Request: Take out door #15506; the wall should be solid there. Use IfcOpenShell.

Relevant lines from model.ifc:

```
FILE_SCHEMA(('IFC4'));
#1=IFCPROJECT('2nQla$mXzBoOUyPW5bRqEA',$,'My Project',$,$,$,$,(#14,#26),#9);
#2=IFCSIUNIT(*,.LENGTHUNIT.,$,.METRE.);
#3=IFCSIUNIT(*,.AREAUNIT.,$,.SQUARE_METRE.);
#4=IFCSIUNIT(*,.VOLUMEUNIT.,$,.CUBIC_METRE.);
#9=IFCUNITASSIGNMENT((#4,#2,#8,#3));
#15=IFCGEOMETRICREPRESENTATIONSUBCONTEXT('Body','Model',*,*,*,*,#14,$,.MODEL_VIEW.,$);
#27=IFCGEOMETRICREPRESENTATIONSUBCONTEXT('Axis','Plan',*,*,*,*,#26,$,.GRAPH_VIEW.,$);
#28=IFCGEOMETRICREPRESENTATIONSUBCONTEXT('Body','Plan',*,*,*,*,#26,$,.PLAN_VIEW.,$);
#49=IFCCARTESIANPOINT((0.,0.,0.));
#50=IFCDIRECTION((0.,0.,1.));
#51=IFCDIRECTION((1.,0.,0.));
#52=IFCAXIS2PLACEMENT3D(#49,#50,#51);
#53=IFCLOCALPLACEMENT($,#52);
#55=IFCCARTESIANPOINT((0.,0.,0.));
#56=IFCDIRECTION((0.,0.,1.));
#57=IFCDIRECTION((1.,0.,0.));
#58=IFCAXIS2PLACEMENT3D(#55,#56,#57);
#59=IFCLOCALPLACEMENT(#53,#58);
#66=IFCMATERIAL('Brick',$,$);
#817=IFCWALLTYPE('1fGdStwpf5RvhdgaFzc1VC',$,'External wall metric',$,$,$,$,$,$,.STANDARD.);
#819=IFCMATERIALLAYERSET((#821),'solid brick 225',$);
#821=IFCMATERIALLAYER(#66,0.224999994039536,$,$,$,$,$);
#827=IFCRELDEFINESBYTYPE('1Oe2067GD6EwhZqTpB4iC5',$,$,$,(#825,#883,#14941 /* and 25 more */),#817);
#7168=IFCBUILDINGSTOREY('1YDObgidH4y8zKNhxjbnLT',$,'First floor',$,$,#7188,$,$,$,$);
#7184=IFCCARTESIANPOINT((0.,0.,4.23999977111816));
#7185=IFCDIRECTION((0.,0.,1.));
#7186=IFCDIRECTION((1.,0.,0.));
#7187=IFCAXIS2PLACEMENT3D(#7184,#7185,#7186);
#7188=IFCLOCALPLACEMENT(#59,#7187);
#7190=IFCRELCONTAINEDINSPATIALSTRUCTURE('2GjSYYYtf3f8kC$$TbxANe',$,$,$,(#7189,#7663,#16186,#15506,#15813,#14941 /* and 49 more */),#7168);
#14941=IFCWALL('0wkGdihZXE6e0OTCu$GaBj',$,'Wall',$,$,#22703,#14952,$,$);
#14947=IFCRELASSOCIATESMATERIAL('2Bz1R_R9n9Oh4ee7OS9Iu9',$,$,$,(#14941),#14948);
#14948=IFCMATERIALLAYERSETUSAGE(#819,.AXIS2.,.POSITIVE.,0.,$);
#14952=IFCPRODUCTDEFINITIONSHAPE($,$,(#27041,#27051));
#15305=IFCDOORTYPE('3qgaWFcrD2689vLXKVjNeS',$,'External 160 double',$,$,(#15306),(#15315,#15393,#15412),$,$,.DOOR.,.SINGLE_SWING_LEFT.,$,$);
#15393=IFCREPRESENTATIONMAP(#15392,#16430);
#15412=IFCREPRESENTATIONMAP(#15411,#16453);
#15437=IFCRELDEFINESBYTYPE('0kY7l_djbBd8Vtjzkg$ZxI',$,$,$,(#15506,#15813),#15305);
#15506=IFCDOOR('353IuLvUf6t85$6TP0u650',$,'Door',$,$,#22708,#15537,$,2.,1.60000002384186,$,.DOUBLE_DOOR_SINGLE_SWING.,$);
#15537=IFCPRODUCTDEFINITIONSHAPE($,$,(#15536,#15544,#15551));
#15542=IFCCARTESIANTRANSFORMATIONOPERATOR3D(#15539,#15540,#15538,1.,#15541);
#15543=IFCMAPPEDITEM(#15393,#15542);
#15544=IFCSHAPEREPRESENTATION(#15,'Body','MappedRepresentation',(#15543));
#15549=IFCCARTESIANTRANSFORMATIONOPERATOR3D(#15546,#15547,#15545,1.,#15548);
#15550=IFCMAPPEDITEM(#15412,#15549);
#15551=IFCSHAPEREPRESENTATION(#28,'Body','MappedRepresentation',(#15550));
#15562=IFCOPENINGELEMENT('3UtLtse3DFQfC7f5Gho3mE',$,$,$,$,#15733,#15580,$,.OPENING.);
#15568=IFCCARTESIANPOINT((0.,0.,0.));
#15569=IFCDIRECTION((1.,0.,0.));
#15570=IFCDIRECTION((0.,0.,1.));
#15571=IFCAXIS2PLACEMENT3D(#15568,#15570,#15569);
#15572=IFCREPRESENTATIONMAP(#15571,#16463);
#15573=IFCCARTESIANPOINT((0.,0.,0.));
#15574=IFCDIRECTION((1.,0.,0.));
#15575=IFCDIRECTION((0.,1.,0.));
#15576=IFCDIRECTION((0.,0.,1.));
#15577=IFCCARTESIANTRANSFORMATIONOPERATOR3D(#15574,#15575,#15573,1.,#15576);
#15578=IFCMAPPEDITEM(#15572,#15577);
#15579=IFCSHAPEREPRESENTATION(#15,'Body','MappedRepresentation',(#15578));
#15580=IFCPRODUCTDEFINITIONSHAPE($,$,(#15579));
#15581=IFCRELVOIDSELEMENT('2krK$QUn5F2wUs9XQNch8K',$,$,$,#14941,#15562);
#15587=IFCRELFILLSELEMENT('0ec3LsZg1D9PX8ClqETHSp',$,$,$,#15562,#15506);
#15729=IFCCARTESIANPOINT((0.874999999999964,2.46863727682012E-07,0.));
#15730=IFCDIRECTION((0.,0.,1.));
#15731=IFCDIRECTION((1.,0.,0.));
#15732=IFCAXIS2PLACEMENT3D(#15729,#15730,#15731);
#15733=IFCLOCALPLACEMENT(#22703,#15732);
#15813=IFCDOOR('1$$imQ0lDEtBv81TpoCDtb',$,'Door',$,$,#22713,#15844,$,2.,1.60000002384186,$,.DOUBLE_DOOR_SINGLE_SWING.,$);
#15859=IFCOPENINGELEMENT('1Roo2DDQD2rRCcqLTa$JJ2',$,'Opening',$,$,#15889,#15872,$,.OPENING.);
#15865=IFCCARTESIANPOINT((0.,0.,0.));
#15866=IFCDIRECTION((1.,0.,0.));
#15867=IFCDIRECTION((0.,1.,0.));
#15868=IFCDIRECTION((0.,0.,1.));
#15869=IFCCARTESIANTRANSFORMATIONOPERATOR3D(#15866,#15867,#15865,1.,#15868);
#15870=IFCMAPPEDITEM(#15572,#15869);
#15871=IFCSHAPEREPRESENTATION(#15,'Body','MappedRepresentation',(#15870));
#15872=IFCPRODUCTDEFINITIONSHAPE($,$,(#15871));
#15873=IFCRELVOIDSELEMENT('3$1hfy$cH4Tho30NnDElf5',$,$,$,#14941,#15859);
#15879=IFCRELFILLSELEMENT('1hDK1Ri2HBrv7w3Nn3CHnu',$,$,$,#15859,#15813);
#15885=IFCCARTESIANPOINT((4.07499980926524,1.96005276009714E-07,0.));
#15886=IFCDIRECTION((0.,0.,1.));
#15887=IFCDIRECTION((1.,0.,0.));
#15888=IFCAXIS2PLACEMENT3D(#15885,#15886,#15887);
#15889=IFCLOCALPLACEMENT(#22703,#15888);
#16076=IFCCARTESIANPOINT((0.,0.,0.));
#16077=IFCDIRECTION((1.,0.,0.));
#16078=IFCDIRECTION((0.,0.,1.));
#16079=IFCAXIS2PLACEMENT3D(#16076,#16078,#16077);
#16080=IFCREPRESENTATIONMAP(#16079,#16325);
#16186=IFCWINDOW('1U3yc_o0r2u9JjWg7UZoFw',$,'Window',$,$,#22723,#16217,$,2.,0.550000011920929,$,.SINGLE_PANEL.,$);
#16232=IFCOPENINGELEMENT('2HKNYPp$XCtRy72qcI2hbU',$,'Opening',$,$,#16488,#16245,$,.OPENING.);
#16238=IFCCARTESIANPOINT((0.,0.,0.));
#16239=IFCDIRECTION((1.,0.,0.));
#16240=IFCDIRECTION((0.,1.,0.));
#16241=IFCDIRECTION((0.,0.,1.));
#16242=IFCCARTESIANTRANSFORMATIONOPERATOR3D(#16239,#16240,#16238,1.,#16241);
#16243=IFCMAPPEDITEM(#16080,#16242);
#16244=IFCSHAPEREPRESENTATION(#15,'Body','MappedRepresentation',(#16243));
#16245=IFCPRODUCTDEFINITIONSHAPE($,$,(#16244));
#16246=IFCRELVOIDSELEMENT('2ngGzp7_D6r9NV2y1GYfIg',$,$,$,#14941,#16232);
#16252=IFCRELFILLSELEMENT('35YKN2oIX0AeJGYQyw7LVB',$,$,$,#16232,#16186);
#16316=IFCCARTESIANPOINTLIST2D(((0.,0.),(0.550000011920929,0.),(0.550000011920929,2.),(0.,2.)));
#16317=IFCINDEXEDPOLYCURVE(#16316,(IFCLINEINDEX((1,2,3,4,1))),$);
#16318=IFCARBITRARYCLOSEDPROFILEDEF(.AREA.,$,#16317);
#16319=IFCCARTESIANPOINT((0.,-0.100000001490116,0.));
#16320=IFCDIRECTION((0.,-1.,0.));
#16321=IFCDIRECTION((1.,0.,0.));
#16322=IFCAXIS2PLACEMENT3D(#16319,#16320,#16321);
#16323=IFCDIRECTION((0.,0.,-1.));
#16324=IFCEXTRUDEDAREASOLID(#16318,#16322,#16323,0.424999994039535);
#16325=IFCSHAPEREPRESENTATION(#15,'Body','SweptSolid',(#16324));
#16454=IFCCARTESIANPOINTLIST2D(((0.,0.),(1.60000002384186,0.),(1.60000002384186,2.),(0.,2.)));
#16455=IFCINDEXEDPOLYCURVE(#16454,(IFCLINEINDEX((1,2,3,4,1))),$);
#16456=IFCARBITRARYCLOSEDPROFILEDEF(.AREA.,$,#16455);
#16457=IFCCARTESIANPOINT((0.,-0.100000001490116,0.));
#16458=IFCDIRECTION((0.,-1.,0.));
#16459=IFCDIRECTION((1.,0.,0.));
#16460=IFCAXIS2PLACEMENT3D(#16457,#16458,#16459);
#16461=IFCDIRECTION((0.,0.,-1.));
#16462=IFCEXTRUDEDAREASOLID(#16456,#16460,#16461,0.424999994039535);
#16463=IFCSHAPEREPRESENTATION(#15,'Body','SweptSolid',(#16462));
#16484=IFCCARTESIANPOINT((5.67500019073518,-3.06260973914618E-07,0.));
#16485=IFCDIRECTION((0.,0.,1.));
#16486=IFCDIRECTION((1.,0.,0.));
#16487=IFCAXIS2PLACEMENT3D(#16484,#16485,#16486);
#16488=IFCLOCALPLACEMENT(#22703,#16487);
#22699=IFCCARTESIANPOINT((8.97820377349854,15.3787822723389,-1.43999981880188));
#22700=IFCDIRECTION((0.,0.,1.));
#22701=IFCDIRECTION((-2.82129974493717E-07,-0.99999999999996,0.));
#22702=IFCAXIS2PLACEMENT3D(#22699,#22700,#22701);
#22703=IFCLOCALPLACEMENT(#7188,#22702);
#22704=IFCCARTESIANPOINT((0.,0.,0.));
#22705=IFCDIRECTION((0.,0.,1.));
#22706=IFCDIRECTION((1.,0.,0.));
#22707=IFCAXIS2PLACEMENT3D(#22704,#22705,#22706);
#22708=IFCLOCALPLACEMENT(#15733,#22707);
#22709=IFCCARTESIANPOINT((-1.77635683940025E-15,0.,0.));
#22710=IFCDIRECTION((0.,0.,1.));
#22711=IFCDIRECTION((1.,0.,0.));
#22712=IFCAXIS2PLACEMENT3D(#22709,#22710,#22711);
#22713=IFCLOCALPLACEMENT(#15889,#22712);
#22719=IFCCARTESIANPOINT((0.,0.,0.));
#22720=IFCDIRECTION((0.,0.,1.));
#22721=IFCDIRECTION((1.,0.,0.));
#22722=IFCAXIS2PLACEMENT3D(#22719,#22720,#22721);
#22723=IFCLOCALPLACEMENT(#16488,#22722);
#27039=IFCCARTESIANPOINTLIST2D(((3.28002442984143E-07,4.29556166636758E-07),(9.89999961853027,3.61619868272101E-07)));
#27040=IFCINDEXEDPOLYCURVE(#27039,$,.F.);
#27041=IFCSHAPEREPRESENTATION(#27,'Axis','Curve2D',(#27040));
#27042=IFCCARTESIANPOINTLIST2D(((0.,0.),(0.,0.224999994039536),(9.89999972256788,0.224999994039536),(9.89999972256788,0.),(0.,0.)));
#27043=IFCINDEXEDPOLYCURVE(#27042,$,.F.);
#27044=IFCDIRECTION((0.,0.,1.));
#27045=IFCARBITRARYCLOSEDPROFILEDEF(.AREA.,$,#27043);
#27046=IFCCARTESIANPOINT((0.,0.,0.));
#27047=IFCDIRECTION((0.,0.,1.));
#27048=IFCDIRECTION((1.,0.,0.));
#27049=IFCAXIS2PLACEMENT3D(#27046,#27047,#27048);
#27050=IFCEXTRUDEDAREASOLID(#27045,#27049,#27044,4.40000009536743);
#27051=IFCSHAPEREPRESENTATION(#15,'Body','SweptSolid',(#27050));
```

```python
import ifcopenshell
import ifcopenshell.api.feature
import ifcopenshell.api.root
import ifcopenshell.geom
import ifcopenshell.util.shape

model = ifcopenshell.open("model.ifc")
settings = ifcopenshell.geom.settings()


def volume(element):
    """Net volume in cubic metres, openings subtracted."""
    shape = ifcopenshell.geom.create_shape(settings, element)
    return ifcopenshell.util.shape.get_volume(shape.geometry)


door = model.by_id(15506)
opening = door.FillsVoids[0].RelatingOpeningElement
wall = opening.VoidsElements[0].RelatingBuildingElement
before = volume(wall)

ifcopenshell.api.root.remove_product(model, product=door)
ifcopenshell.api.feature.remove_feature(model, feature=opening)

after = volume(wall)

print(f"wall volume {before:.3f} -> {after:.3f} m3")

model.write("model_updated.ifc")
```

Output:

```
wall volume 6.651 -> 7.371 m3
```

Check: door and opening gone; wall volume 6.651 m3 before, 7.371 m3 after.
